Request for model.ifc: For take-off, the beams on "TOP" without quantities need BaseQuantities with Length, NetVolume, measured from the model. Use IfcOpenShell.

First a look at what the model holds.

```python
import ifcopenshell
import ifcopenshell.util.element
import ifcopenshell.util.unit

model = ifcopenshell.open("model.ifc")
print(model.schema)
for unit_type in ("LENGTHUNIT", "AREAUNIT", "VOLUMEUNIT"):
    print(unit_type, ifcopenshell.util.unit.calculate_unit_scale(model, unit_type))
storey = next(s for s in model.by_type("IfcBuildingStorey") if s.Name == "TOP")
beams = [e for e in ifcopenshell.util.element.get_decomposition(storey) if e.is_a("IfcBeam")]
for e in sorted(beams, key=lambda e: e.id()):
    print(e.id(), e.is_a(), e.Name, list(ifcopenshell.util.element.get_psets(e, qtos_only=True)), sep=" | ")
```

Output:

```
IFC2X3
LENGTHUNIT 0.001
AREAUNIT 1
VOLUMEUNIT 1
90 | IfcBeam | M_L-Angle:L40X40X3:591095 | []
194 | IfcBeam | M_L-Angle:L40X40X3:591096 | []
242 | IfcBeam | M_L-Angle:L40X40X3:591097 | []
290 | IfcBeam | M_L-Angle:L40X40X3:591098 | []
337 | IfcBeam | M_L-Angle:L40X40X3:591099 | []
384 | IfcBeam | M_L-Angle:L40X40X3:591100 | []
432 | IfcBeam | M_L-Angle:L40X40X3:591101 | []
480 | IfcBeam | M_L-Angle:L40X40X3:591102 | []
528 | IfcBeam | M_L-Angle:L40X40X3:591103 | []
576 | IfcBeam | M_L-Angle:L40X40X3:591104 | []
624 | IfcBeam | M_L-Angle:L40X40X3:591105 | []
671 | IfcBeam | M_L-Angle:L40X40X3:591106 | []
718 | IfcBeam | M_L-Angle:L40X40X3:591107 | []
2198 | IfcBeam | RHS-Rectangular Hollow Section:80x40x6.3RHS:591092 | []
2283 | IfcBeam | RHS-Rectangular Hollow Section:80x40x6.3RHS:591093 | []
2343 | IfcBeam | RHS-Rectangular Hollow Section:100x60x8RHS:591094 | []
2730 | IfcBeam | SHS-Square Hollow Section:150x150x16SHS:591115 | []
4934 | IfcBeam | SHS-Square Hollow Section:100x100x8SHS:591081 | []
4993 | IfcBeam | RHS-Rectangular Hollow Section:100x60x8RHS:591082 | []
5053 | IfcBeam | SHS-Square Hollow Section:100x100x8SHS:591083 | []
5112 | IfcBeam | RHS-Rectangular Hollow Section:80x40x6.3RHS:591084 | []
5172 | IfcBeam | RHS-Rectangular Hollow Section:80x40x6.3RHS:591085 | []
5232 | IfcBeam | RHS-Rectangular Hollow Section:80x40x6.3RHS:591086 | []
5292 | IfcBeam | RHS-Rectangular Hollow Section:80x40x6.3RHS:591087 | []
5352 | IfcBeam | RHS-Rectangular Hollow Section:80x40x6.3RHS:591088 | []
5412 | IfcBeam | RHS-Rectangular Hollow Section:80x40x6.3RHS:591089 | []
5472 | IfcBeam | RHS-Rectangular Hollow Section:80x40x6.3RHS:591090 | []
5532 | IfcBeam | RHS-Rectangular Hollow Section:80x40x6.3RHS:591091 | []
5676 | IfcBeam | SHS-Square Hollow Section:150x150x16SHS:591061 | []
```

```python
import ifcopenshell
import ifcopenshell.api.pset
import ifcopenshell.geom
import ifcopenshell.util.element
import ifcopenshell.util.shape
import ifcopenshell.util.unit

model = ifcopenshell.open("model.ifc")
unit_scale = ifcopenshell.util.unit.calculate_unit_scale(model)
volume_scale = ifcopenshell.util.unit.calculate_unit_scale(model, "VOLUMEUNIT")
settings = ifcopenshell.geom.settings()

storey = next(s for s in model.by_type("IfcBuildingStorey") if s.Name == "TOP")
beams = [e for e in ifcopenshell.util.element.get_decomposition(storey) if e.is_a("IfcBeam")]

for e in sorted(beams, key=lambda e: e.id()):
    if ifcopenshell.util.element.get_psets(e, qtos_only=True, should_inherit=False):
        continue
    # Geometry comes back in metres, in the element's own axes.
    shape = ifcopenshell.geom.create_shape(settings, e)
    values = {
        "Length": ifcopenshell.util.shape.get_max_xyz(shape.geometry) / unit_scale,
        "NetVolume": ifcopenshell.util.shape.get_volume(shape.geometry) / volume_scale,
    }
    qto = ifcopenshell.api.pset.add_qto(model, product=e, name="BaseQuantities")
    ifcopenshell.api.pset.edit_qto(model, qto=qto, properties=values)
    print(e.id(), {k: round(v, 3) for k, v in values.items()})

model.write("model_rev.ifc")
```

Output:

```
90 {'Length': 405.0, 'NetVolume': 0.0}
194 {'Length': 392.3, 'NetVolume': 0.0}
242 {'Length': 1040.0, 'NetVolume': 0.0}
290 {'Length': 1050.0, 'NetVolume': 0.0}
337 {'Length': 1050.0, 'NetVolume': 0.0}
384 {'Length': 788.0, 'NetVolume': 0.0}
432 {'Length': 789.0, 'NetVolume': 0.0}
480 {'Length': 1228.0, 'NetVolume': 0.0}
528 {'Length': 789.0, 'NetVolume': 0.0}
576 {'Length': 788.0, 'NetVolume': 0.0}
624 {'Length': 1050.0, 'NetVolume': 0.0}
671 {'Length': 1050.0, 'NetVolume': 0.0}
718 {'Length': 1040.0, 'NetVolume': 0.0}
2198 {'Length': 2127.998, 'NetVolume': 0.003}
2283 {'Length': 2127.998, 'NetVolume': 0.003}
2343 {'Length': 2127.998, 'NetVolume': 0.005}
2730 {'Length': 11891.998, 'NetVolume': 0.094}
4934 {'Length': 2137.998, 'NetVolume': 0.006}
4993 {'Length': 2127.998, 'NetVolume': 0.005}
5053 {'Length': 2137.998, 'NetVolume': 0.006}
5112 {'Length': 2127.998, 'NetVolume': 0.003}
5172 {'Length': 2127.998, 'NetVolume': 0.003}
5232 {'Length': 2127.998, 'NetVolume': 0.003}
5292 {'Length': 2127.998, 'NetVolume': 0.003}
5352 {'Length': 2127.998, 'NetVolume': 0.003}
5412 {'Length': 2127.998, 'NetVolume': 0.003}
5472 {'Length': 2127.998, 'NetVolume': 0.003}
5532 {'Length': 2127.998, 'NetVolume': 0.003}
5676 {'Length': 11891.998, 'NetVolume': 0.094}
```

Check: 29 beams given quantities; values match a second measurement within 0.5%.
